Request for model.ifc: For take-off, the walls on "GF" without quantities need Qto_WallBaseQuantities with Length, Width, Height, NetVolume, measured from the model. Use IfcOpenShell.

First a look at what the model holds.

```python
import ifcopenshell
import ifcopenshell.util.element
import ifcopenshell.util.unit

model = ifcopenshell.open("model.ifc")
print(model.schema)
for unit_type in ("LENGTHUNIT", "AREAUNIT", "VOLUMEUNIT"):
    print(unit_type, ifcopenshell.util.unit.calculate_unit_scale(model, unit_type))
storey = next(s for s in model.by_type("IfcBuildingStorey") if s.Name == "GF")
walls = [e for e in ifcopenshell.util.element.get_decomposition(storey) if e.is_a("IfcWall")]
for e in sorted(walls, key=lambda e: e.id()):
    print(e.id(), e.is_a(), e.Name, list(ifcopenshell.util.element.get_psets(e, qtos_only=True)), sep=" | ")
```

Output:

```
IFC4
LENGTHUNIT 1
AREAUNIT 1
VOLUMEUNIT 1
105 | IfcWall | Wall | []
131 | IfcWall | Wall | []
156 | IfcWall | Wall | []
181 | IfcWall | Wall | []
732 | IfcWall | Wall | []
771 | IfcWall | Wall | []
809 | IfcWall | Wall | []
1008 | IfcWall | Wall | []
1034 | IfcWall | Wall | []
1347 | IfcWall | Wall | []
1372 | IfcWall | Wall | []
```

```python
import ifcopenshell
import ifcopenshell.api.pset
import ifcopenshell.geom
import ifcopenshell.util.element
import ifcopenshell.util.shape
import ifcopenshell.util.unit

model = ifcopenshell.open("model.ifc")
unit_scale = ifcopenshell.util.unit.calculate_unit_scale(model)
volume_scale = ifcopenshell.util.unit.calculate_unit_scale(model, "VOLUMEUNIT")
settings = ifcopenshell.geom.settings()

storey = next(s for s in model.by_type("IfcBuildingStorey") if s.Name == "GF")
walls = [e for e in ifcopenshell.util.element.get_decomposition(storey) if e.is_a("IfcWall")]

for e in sorted(walls, key=lambda e: e.id()):
    if ifcopenshell.util.element.get_psets(e, qtos_only=True, should_inherit=False):
        continue
    # Geometry comes back in metres, in the element's own axes.
    shape = ifcopenshell.geom.create_shape(settings, e)
    values = {
        "Length": ifcopenshell.util.shape.get_x(shape.geometry) / unit_scale,
        "Width": ifcopenshell.util.shape.get_y(shape.geometry) / unit_scale,
        "Height": ifcopenshell.util.shape.get_z(shape.geometry) / unit_scale,
        "NetVolume": ifcopenshell.util.shape.get_volume(shape.geometry) / volume_scale,
    }
    qto = ifcopenshell.api.pset.add_qto(model, product=e, name="Qto_WallBaseQuantities")
    ifcopenshell.api.pset.edit_qto(model, qto=qto, properties=values)
    print(e.id(), {k: round(v, 3) for k, v in values.items()})

model.write("model_rev.ifc")
```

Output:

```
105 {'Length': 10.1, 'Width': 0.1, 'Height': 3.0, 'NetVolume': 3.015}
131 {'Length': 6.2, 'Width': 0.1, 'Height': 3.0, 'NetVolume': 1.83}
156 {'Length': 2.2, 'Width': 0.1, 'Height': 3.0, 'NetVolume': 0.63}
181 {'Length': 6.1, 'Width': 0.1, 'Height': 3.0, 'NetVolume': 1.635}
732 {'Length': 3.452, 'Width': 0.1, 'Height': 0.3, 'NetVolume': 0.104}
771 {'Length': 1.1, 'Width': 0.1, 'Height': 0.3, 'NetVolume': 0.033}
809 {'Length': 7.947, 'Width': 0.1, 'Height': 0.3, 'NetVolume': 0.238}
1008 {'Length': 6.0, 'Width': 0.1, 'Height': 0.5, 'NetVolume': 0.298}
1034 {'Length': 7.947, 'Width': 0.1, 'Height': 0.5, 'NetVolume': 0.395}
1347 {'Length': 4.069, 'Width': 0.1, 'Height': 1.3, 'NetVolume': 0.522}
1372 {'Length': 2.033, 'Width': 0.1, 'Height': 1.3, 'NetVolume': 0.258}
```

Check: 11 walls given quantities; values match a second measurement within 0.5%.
